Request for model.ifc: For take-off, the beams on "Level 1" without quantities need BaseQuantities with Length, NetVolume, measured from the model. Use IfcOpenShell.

First a look at what the model holds.

```python
import ifcopenshell
import ifcopenshell.util.element
import ifcopenshell.util.unit

model = ifcopenshell.open("model.ifc")
print(model.schema)
for unit_type in ("LENGTHUNIT", "AREAUNIT", "VOLUMEUNIT"):
    print(unit_type, ifcopenshell.util.unit.calculate_unit_scale(model, unit_type))
storey = next(s for s in model.by_type("IfcBuildingStorey") if s.Name == "Level 1")
beams = [e for e in ifcopenshell.util.element.get_decomposition(storey) if e.is_a("IfcBeam")]
for e in sorted(beams, key=lambda e: e.id()):
    print(e.id(), e.is_a(), e.Name, list(ifcopenshell.util.element.get_psets(e, qtos_only=True)), sep=" | ")
```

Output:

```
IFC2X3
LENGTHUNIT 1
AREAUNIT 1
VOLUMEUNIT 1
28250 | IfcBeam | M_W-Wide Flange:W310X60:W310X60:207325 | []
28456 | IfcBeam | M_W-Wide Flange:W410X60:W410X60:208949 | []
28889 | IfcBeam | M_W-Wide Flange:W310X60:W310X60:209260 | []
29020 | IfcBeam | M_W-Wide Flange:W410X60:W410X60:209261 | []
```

```python
import ifcopenshell
import ifcopenshell.api.pset
import ifcopenshell.geom
import ifcopenshell.util.element
import ifcopenshell.util.shape
import ifcopenshell.util.unit

model = ifcopenshell.open("model.ifc")
unit_scale = ifcopenshell.util.unit.calculate_unit_scale(model)
volume_scale = ifcopenshell.util.unit.calculate_unit_scale(model, "VOLUMEUNIT")
settings = ifcopenshell.geom.settings()

storey = next(s for s in model.by_type("IfcBuildingStorey") if s.Name == "Level 1")
beams = [e for e in ifcopenshell.util.element.get_decomposition(storey) if e.is_a("IfcBeam")]

for e in sorted(beams, key=lambda e: e.id()):
    if ifcopenshell.util.element.get_psets(e, qtos_only=True, should_inherit=False):
        continue
    # Geometry comes back in metres, in the element's own axes.
    shape = ifcopenshell.geom.create_shape(settings, e)
    values = {
        "Length": ifcopenshell.util.shape.get_max_xyz(shape.geometry) / unit_scale,
        "NetVolume": ifcopenshell.util.shape.get_volume(shape.geometry) / volume_scale,
    }
    qto = ifcopenshell.api.pset.add_qto(model, product=e, name="BaseQuantities")
    ifcopenshell.api.pset.edit_qto(model, qto=qto, properties=values)
    print(e.id(), {k: round(v, 3) for k, v in values.items()})

model.write("model_rev.ifc")
```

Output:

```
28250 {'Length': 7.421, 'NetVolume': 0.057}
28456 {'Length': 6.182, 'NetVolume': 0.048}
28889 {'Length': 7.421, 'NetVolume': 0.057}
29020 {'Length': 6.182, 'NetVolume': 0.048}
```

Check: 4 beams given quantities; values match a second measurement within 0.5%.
